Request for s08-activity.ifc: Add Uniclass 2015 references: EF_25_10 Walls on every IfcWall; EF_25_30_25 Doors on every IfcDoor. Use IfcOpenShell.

First a look at what the model holds.

```python
import ifcopenshell

model = ifcopenshell.open("s08-activity.ifc")
print(model.schema)
print("classifications:", [c.Name for c in model.by_type("IfcClassification")])
for ifc_class in ("IfcDoor", "IfcRoof", "IfcStair", "IfcWall", "IfcWindow"):
    print(ifc_class, len(model.by_type(ifc_class)))
```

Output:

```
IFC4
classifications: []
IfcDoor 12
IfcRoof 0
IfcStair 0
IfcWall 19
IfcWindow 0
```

```python
import ifcopenshell
import ifcopenshell.api.classification

model = ifcopenshell.open("s08-activity.ifc")

system = ifcopenshell.api.classification.add_classification(model, classification="Uniclass 2015")

codes = {
    "IfcWall": ("EF_25_10", "Walls"),
    "IfcDoor": ("EF_25_30_25", "Doors"),
}
for ifc_class, (code, name) in codes.items():
    products = model.by_type(ifc_class)
    ifcopenshell.api.classification.add_reference(
        model, products=products, classification=system, identification=code, name=name
    )
    print(code, len(products))

model.write("s08-activity_rev.ifc")
```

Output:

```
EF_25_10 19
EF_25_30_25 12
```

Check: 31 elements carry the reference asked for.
